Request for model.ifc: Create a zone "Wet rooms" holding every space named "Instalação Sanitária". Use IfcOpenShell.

First a look at what the model holds.

```python
import ifcopenshell

model = ifcopenshell.open("model.ifc")
print(model.schema)
seen = {}
for space in model.by_type("IfcSpace"):
    seen[space.LongName] = seen.get(space.LongName, 0) + 1
for name, count in sorted(seen.items(), key=str):
    print(count, "x", name)
print("zones:", [z.Name for z in model.by_type("IfcZone")][:20])
```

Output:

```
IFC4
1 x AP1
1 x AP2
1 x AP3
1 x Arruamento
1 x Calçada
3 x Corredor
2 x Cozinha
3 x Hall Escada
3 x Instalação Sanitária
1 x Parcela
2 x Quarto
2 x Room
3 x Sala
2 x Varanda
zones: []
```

```python
import ifcopenshell
import ifcopenshell.api.group
import ifcopenshell.api.root

model = ifcopenshell.open("model.ifc")

names = {"Instalação Sanitária"}
spaces = [s for s in model.by_type("IfcSpace") if s.LongName in names]

zone = ifcopenshell.api.root.create_entity(model, ifc_class="IfcZone", name="Wet rooms")
ifcopenshell.api.group.assign_group(model, products=spaces, group=zone)
print(len(spaces), "spaces in", zone.Name)

model.write("model_v2.ifc")
```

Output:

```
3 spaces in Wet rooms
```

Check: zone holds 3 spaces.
